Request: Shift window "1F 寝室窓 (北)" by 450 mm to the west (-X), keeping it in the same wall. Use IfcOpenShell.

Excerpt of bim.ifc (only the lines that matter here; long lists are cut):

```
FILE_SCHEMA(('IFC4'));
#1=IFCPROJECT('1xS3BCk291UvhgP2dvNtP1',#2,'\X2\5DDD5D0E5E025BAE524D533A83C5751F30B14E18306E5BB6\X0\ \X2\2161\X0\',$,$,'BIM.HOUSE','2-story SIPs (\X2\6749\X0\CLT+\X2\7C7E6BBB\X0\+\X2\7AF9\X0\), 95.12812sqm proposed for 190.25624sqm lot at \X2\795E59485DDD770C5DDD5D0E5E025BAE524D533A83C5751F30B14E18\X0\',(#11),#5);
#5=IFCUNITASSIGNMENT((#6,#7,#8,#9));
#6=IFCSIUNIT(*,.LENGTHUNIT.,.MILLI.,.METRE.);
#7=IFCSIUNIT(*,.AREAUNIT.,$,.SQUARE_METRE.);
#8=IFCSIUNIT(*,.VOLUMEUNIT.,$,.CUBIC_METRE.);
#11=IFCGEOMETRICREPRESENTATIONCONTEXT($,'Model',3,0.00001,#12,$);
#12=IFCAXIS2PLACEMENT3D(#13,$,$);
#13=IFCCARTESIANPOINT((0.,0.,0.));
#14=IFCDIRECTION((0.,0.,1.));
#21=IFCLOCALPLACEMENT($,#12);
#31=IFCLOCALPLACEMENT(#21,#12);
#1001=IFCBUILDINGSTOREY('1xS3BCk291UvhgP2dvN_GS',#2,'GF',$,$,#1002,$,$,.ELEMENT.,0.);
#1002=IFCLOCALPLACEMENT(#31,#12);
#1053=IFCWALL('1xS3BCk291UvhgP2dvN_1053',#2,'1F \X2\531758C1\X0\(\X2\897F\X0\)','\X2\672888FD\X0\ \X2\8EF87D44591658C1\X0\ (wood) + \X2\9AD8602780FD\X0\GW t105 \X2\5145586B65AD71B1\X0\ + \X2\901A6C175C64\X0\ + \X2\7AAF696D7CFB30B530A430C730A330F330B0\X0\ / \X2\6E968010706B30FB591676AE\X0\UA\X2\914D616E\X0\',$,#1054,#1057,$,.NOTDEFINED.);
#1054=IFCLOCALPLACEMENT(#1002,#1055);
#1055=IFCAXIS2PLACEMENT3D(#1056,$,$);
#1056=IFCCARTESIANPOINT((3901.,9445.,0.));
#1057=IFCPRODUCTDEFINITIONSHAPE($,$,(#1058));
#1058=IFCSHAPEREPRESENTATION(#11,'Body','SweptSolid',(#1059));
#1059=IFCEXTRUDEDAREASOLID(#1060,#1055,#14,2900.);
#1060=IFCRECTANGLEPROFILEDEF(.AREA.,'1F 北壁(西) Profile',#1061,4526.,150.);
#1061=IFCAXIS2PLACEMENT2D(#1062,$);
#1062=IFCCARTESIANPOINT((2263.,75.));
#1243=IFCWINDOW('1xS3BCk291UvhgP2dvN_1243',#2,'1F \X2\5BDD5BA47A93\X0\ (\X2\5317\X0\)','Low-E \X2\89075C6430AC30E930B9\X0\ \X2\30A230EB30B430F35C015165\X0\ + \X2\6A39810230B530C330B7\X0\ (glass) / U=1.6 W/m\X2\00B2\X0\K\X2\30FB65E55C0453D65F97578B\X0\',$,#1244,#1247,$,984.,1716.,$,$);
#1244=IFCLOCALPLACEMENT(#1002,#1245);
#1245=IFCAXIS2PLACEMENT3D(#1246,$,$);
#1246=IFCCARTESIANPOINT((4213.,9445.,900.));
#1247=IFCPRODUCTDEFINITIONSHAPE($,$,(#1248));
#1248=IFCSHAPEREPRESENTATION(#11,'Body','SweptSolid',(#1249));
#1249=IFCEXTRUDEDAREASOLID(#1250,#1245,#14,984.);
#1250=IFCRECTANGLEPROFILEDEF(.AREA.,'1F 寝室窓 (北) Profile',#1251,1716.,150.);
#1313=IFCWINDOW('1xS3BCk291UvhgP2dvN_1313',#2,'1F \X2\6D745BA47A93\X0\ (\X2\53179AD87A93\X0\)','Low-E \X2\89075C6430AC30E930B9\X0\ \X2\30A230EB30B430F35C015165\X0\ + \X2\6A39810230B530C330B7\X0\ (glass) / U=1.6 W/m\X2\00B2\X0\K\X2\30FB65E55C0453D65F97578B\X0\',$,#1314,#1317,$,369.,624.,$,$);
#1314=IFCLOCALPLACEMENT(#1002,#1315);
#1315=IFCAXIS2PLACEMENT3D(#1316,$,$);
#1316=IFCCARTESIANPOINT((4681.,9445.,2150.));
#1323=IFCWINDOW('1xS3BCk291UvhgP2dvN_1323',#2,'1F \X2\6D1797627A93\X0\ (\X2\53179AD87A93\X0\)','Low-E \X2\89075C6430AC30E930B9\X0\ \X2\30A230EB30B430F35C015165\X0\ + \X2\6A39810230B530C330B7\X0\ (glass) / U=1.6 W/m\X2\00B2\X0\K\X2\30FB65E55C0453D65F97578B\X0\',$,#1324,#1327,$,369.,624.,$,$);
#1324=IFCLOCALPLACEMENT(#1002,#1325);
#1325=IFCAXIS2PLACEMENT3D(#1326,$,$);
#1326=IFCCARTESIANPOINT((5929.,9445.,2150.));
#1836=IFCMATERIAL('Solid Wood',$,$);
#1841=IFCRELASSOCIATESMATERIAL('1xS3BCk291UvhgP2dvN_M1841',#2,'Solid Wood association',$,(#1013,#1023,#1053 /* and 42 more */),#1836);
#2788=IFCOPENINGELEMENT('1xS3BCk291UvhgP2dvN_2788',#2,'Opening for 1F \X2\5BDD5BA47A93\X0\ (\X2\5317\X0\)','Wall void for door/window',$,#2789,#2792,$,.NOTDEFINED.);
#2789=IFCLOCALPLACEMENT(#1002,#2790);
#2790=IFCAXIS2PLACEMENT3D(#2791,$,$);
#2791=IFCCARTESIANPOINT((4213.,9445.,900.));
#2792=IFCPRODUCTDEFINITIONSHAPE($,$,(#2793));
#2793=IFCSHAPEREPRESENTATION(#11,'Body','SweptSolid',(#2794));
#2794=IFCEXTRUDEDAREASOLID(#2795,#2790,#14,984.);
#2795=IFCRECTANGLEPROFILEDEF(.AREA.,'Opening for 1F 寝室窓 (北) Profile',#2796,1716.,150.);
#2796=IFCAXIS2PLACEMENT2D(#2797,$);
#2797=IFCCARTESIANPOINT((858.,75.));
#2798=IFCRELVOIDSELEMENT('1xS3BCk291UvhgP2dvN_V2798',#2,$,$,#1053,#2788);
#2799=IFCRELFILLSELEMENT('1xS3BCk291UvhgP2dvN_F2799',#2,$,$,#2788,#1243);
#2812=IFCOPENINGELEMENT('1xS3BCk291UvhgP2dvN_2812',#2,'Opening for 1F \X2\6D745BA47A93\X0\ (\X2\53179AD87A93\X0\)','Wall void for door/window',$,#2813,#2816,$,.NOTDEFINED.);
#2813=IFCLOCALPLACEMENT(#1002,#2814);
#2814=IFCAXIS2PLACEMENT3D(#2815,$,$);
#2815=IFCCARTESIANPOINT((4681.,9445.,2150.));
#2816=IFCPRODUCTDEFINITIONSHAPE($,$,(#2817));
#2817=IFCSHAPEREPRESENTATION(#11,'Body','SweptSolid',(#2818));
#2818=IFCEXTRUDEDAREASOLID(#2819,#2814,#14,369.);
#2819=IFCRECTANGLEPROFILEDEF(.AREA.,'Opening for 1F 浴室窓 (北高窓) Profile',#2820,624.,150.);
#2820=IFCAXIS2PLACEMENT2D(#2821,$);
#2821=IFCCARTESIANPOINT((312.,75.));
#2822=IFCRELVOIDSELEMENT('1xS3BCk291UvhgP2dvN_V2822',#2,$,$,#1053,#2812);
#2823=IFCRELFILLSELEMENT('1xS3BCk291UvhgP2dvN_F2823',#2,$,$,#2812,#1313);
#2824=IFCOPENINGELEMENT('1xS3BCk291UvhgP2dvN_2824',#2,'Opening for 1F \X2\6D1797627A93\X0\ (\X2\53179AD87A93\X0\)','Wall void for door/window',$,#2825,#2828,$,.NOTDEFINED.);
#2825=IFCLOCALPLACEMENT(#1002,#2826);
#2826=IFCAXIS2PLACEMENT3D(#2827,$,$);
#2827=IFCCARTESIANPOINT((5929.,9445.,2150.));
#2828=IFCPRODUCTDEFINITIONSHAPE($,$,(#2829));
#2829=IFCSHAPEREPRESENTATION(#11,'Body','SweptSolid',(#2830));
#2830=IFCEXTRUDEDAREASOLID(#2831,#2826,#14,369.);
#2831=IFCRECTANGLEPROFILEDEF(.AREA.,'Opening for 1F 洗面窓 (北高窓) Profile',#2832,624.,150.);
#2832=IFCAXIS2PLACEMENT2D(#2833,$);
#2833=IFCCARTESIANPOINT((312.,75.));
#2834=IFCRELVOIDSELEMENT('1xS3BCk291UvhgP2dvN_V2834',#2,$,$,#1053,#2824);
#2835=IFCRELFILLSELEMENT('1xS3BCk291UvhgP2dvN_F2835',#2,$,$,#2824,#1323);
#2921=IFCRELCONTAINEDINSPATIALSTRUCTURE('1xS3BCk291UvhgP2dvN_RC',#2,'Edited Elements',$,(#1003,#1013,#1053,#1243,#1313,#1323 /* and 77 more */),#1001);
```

```python
import ifcopenshell
import ifcopenshell.api.geometry
import ifcopenshell.util.placement
import ifcopenshell.util.unit

model = ifcopenshell.open("bim.ifc")
unit_scale = ifcopenshell.util.unit.calculate_unit_scale(model)

window = model.by_guid("1xS3BCk291UvhgP2dvN_1243")
opening = window.FillsVoids[0].RelatingOpeningElement
wall = opening.VoidsElements[0].RelatingBuildingElement

wall_matrix = ifcopenshell.util.placement.get_local_placement(wall.ObjectPlacement)
shift = wall_matrix[:3, 0] * -0.45 / unit_scale
before = ifcopenshell.util.placement.get_local_placement(window.ObjectPlacement)[:3, 3].copy()

# The window is not placed relative to its opening, so move both.
for product in (opening, window):
    matrix = ifcopenshell.util.placement.get_local_placement(product.ObjectPlacement)
    matrix[:3, 3] += shift
    ifcopenshell.api.geometry.edit_object_placement(model, product=product, matrix=matrix, is_si=False)

after = ifcopenshell.util.placement.get_local_placement(window.ObjectPlacement)[:3, 3]
print("window moved by", (after - before).round(3) + 0.0)

model.write("bim_edited.ifc")
```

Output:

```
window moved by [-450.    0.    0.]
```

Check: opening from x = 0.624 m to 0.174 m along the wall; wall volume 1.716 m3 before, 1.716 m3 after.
